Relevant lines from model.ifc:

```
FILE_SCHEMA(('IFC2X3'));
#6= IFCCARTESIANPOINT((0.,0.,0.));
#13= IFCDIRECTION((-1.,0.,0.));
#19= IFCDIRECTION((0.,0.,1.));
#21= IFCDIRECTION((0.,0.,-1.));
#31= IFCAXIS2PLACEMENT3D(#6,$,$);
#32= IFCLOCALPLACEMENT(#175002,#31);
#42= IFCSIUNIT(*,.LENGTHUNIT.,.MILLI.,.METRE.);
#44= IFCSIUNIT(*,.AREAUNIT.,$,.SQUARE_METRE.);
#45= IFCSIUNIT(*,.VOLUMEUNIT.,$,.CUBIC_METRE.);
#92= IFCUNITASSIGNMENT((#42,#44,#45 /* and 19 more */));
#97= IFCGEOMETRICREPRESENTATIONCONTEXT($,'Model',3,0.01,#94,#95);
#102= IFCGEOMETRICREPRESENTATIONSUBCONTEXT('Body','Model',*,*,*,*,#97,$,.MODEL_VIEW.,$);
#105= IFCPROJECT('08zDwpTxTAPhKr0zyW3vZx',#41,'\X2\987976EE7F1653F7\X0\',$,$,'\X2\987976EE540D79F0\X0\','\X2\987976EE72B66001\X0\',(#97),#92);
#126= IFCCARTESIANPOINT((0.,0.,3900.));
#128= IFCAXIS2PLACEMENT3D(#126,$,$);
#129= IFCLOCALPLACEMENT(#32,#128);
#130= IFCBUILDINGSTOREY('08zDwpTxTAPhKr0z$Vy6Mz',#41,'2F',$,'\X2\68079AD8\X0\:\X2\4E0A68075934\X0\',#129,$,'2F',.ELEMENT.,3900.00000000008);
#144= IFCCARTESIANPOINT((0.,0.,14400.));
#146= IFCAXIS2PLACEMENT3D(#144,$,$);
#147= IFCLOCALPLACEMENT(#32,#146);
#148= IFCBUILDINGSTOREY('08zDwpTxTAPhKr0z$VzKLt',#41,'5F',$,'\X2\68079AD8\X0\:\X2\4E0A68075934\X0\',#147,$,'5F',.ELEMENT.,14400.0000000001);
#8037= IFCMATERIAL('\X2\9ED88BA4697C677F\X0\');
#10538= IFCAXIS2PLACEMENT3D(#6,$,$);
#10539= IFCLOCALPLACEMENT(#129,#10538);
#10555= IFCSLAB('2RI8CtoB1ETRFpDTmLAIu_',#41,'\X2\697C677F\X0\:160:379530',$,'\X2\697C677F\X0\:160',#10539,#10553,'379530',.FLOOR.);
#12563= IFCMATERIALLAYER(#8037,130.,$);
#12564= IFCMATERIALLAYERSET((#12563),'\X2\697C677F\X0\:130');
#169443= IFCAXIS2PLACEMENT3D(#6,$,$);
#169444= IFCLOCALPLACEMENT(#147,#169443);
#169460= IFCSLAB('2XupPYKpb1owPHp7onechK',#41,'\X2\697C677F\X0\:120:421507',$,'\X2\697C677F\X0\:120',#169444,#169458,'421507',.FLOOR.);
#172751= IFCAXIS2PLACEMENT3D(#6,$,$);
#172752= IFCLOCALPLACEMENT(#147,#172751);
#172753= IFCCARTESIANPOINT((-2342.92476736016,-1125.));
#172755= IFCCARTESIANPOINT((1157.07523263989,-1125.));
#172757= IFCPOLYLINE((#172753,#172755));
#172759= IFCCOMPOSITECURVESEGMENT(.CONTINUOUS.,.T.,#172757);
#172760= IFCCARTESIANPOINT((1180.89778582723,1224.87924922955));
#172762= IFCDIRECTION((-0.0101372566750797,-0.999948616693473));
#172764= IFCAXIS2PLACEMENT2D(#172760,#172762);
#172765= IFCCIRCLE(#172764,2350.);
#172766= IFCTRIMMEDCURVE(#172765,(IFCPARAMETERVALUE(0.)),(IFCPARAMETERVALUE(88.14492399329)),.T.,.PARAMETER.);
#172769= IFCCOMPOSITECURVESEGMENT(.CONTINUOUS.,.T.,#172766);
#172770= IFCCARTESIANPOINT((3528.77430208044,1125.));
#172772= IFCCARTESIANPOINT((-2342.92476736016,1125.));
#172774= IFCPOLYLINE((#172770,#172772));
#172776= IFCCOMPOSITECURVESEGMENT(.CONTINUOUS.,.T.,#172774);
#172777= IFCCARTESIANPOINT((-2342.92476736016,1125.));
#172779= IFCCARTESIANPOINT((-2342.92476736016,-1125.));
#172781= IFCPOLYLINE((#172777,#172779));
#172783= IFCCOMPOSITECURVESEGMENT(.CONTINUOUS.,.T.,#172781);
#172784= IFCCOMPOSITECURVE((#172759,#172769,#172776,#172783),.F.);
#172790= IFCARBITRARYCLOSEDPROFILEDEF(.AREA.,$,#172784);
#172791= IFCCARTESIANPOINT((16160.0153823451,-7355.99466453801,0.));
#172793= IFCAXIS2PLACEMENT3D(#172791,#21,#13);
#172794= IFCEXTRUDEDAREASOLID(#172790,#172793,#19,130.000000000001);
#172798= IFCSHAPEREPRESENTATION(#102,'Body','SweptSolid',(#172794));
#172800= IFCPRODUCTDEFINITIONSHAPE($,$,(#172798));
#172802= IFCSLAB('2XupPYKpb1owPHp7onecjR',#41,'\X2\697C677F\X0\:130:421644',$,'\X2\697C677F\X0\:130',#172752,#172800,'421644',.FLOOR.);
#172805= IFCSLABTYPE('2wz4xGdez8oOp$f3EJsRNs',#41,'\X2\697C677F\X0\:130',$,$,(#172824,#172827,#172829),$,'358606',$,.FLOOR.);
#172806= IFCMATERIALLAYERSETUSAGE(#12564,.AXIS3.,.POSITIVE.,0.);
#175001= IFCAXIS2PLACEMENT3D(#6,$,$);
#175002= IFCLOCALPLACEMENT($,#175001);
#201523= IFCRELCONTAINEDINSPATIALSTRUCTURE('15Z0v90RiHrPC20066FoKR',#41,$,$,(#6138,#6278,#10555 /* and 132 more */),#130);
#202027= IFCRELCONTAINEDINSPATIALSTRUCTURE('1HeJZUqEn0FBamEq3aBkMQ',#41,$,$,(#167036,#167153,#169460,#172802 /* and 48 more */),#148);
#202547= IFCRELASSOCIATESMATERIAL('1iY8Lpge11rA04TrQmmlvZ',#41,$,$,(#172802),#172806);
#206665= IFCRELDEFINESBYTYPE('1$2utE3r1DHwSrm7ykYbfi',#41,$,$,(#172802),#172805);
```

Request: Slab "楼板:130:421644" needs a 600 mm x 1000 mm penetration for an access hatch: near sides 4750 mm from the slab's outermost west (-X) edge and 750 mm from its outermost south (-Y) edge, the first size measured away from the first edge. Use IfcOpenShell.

```python
import numpy as np
import ifcopenshell
import ifcopenshell.api.feature
import ifcopenshell.api.geometry
import ifcopenshell.api.root
import ifcopenshell.geom
import ifcopenshell.util.placement
import ifcopenshell.util.representation
import ifcopenshell.util.shape
import ifcopenshell.util.unit

model = ifcopenshell.open("model.ifc")
unit_scale = ifcopenshell.util.unit.calculate_unit_scale(model)
settings = ifcopenshell.geom.settings()


def volume(element):
    """Net volume in cubic metres, openings subtracted."""
    shape = ifcopenshell.geom.create_shape(settings, element)
    return ifcopenshell.util.shape.get_volume(shape.geometry)


slab = model.by_guid("2XupPYKpb1owPHp7onecjR")
before = volume(slab)

# Extent in the slab's own axes, in metres. The edges named are its -X and -Y sides.
slab_shape = ifcopenshell.geom.create_shape(settings, slab)
vertices = ifcopenshell.util.shape.get_vertices(slab_shape.geometry)
x_min, y_min, bottom = vertices.min(axis=0)
top = vertices[:, 2].max()

opening = ifcopenshell.api.root.create_entity(model, ifc_class="IfcOpeningElement", name="Access hatch opening")
context = ifcopenshell.util.representation.get_context(model, "Model", "Body", "MODEL_VIEW")
width, depth = 0.6, 1
outline = [(0.0, 0.0), (width, 0.0), (width, depth), (0.0, depth), (0.0, 0.0)]
# Overshoot both faces by 50 mm so the cut is clean.
shape = ifcopenshell.api.geometry.add_slab_representation(
    model, context=context, depth=top - bottom + 0.1, polyline=outline
)
ifcopenshell.api.geometry.assign_representation(model, product=opening, representation=shape)

matrix = ifcopenshell.util.placement.get_local_placement(slab.ObjectPlacement)
matrix[:, 3] = matrix @ np.append(np.array([x_min + 4.75, y_min + 0.75, bottom - 0.05]) / unit_scale, 1.0)
ifcopenshell.api.geometry.edit_object_placement(model, product=opening, matrix=matrix, is_si=False)
ifcopenshell.api.feature.add_feature(model, feature=opening, element=slab)

after = volume(slab)

print(f"slab volume {before:.3f} -> {after:.3f} m3")

model.write("model_v2.ifc")
```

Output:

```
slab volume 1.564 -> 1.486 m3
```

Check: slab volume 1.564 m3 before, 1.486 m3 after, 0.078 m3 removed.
